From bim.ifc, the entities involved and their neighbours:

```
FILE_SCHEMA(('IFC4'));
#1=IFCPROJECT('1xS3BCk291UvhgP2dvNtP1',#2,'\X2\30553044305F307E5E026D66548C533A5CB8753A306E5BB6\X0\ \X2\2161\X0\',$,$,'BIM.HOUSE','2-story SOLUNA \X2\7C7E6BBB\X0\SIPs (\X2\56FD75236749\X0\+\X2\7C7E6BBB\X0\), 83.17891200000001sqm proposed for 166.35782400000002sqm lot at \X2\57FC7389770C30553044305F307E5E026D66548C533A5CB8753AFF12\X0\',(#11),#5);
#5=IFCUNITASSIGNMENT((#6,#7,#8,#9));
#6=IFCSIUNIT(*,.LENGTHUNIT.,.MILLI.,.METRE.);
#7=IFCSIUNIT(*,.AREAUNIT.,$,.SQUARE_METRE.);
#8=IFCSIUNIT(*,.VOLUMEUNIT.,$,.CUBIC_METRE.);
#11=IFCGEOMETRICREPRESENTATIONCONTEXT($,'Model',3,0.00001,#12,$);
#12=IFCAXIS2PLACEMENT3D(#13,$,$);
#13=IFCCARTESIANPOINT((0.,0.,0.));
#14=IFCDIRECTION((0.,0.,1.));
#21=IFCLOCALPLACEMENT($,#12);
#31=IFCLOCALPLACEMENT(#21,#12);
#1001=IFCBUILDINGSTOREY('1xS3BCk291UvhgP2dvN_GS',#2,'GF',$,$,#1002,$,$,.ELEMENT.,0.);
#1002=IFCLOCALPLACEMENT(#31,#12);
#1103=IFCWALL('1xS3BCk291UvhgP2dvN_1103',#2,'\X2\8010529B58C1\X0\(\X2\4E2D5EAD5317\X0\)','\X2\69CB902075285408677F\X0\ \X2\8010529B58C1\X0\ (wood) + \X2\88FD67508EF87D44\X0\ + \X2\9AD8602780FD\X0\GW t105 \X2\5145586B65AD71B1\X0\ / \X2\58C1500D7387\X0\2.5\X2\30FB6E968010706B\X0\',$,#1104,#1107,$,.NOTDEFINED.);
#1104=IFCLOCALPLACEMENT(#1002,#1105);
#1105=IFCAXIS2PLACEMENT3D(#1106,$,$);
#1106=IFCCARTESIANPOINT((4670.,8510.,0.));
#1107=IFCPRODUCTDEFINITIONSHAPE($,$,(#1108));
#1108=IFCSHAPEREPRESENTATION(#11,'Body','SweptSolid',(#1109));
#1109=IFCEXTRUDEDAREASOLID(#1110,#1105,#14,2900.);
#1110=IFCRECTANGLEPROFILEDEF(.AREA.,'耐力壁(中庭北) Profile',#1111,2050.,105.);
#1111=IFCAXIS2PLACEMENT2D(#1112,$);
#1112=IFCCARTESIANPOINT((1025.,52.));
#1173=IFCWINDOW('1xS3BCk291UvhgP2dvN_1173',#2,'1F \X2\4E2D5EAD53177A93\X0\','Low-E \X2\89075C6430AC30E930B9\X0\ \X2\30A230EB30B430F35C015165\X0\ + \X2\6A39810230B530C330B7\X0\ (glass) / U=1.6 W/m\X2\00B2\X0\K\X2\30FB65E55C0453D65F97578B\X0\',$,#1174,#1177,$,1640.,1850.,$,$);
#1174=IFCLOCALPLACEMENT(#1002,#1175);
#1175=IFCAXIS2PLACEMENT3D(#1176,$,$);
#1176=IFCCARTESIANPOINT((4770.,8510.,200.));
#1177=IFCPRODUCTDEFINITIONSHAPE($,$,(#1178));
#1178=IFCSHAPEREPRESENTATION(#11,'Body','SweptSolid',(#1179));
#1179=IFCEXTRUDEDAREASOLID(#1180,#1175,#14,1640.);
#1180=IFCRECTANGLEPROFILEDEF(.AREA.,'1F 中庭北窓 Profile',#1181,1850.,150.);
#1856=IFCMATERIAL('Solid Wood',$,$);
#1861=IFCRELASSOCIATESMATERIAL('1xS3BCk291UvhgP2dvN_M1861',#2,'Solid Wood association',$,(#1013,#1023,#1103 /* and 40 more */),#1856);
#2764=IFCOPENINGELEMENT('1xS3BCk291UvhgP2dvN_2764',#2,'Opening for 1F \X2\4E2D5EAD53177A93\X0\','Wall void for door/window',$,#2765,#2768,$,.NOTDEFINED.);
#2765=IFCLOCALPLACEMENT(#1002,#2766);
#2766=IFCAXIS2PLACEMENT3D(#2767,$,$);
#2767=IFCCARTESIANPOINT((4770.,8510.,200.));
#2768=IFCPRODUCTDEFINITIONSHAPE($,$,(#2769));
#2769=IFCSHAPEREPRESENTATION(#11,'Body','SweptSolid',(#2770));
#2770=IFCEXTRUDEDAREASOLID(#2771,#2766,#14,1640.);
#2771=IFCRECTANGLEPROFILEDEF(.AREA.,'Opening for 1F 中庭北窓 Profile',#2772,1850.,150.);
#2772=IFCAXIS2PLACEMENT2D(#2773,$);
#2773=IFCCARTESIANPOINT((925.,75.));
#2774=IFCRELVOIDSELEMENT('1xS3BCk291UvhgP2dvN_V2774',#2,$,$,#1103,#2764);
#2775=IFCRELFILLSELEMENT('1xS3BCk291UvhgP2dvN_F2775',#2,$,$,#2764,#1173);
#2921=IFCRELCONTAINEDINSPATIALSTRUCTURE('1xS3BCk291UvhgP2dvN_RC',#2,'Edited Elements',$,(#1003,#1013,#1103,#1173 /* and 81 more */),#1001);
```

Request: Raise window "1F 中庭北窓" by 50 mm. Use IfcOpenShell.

```python
import numpy as np
import ifcopenshell
import ifcopenshell.api.geometry
import ifcopenshell.util.placement
import ifcopenshell.util.unit

model = ifcopenshell.open("bim.ifc")
unit_scale = ifcopenshell.util.unit.calculate_unit_scale(model)

window = model.by_guid("1xS3BCk291UvhgP2dvN_1173")
opening = window.FillsVoids[0].RelatingOpeningElement
dz = 0.05 / unit_scale

shift = np.array([0.0, 0.0, dz])
# The window is not placed relative to its opening, so move both.
for product in (opening, window):
    matrix = ifcopenshell.util.placement.get_local_placement(product.ObjectPlacement)
    matrix[:3, 3] += shift
    ifcopenshell.api.geometry.edit_object_placement(model, product=product, matrix=matrix, is_si=False)

print(f"moved by {dz * unit_scale:+.3f} m")

model.write("bim_edited.ifc")
```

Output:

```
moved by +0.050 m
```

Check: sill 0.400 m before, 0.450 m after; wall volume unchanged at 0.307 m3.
